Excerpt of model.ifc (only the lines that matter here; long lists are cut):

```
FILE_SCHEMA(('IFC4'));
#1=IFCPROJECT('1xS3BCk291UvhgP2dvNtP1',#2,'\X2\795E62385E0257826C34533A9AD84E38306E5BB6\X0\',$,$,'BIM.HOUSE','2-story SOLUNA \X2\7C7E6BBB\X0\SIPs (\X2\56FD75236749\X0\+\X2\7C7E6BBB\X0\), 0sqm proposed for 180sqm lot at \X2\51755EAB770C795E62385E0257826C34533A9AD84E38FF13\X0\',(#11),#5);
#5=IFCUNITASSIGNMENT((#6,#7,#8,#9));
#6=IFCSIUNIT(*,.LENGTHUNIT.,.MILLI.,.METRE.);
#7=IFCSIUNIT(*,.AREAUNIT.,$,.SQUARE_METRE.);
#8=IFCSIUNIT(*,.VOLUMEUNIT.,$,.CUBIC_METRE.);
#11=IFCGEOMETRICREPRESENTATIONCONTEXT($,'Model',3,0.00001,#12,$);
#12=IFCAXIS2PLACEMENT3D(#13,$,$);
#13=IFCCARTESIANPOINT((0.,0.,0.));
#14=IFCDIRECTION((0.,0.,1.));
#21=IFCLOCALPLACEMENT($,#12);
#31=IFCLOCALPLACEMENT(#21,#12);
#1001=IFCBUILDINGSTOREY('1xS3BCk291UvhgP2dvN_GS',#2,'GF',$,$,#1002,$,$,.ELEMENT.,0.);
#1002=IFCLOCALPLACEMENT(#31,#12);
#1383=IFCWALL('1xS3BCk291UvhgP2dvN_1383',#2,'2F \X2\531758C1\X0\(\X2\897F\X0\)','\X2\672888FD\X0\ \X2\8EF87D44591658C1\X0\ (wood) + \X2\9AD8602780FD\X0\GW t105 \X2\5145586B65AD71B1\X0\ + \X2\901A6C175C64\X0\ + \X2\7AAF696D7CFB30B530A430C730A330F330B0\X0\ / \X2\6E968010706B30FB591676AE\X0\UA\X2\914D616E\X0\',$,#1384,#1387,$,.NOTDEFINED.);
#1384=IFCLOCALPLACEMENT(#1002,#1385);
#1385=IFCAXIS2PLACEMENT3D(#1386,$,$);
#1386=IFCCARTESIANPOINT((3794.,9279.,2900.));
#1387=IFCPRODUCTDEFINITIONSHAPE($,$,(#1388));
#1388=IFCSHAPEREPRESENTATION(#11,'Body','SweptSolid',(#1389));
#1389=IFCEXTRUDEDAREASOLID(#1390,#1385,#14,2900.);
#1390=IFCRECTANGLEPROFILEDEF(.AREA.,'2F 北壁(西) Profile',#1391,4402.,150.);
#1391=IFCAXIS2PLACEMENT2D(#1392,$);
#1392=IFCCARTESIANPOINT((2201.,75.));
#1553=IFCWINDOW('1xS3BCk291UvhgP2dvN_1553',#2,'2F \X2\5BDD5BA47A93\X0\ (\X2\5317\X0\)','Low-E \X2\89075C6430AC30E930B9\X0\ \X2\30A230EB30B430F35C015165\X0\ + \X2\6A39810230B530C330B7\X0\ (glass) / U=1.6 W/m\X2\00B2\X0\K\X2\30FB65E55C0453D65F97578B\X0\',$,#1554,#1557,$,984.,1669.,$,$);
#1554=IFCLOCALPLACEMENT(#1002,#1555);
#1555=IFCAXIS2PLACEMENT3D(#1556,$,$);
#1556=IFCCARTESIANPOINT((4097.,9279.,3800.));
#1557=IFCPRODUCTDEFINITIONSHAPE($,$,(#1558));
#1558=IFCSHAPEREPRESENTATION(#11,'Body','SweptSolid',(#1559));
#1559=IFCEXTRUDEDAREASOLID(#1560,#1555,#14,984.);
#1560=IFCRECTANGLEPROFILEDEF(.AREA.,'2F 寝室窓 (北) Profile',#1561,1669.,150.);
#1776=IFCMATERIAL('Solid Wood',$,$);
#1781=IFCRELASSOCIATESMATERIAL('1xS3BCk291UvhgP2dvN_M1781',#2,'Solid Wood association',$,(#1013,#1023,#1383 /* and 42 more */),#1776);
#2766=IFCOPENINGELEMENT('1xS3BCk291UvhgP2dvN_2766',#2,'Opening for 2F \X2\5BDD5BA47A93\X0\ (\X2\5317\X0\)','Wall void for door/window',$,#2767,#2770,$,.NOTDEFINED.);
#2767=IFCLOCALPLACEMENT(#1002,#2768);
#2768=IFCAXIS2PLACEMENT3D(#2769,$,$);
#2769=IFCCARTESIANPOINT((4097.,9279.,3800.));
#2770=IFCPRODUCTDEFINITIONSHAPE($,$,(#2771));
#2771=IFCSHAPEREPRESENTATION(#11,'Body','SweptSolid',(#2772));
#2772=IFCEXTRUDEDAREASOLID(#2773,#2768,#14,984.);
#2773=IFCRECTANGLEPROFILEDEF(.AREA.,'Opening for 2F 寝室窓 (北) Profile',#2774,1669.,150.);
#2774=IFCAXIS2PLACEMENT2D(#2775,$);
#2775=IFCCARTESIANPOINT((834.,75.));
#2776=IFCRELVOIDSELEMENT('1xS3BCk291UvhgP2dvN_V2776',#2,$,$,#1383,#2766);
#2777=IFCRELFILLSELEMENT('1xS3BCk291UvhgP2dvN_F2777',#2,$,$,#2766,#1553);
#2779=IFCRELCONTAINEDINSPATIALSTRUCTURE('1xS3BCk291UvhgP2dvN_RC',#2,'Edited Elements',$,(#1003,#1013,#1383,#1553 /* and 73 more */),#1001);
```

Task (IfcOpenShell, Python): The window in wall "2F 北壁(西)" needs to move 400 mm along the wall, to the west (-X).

```python
import ifcopenshell
import ifcopenshell.api.geometry
import ifcopenshell.util.placement

model = ifcopenshell.open("model.ifc")

window = model.by_guid("1xS3BCk291UvhgP2dvN_1553")
opening = window.FillsVoids[0].RelatingOpeningElement
wall = opening.VoidsElements[0].RelatingBuildingElement

wall_matrix = ifcopenshell.util.placement.get_local_placement(wall.ObjectPlacement)
shift = wall_matrix[:3, 0] * -400.0
before = ifcopenshell.util.placement.get_local_placement(window.ObjectPlacement)[:3, 3].copy()

# The window is not placed relative to its opening, so move both.
for product in (opening, window):
    matrix = ifcopenshell.util.placement.get_local_placement(product.ObjectPlacement)
    matrix[:3, 3] += shift
    ifcopenshell.api.geometry.edit_object_placement(model, product=product, matrix=matrix, is_si=False)

after = ifcopenshell.util.placement.get_local_placement(window.ObjectPlacement)[:3, 3]
print("window moved by", (after - before).round(3) + 0.0)

model.write("model_v2.ifc")
```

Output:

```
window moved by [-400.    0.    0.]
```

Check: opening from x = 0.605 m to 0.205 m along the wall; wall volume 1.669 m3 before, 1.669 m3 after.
